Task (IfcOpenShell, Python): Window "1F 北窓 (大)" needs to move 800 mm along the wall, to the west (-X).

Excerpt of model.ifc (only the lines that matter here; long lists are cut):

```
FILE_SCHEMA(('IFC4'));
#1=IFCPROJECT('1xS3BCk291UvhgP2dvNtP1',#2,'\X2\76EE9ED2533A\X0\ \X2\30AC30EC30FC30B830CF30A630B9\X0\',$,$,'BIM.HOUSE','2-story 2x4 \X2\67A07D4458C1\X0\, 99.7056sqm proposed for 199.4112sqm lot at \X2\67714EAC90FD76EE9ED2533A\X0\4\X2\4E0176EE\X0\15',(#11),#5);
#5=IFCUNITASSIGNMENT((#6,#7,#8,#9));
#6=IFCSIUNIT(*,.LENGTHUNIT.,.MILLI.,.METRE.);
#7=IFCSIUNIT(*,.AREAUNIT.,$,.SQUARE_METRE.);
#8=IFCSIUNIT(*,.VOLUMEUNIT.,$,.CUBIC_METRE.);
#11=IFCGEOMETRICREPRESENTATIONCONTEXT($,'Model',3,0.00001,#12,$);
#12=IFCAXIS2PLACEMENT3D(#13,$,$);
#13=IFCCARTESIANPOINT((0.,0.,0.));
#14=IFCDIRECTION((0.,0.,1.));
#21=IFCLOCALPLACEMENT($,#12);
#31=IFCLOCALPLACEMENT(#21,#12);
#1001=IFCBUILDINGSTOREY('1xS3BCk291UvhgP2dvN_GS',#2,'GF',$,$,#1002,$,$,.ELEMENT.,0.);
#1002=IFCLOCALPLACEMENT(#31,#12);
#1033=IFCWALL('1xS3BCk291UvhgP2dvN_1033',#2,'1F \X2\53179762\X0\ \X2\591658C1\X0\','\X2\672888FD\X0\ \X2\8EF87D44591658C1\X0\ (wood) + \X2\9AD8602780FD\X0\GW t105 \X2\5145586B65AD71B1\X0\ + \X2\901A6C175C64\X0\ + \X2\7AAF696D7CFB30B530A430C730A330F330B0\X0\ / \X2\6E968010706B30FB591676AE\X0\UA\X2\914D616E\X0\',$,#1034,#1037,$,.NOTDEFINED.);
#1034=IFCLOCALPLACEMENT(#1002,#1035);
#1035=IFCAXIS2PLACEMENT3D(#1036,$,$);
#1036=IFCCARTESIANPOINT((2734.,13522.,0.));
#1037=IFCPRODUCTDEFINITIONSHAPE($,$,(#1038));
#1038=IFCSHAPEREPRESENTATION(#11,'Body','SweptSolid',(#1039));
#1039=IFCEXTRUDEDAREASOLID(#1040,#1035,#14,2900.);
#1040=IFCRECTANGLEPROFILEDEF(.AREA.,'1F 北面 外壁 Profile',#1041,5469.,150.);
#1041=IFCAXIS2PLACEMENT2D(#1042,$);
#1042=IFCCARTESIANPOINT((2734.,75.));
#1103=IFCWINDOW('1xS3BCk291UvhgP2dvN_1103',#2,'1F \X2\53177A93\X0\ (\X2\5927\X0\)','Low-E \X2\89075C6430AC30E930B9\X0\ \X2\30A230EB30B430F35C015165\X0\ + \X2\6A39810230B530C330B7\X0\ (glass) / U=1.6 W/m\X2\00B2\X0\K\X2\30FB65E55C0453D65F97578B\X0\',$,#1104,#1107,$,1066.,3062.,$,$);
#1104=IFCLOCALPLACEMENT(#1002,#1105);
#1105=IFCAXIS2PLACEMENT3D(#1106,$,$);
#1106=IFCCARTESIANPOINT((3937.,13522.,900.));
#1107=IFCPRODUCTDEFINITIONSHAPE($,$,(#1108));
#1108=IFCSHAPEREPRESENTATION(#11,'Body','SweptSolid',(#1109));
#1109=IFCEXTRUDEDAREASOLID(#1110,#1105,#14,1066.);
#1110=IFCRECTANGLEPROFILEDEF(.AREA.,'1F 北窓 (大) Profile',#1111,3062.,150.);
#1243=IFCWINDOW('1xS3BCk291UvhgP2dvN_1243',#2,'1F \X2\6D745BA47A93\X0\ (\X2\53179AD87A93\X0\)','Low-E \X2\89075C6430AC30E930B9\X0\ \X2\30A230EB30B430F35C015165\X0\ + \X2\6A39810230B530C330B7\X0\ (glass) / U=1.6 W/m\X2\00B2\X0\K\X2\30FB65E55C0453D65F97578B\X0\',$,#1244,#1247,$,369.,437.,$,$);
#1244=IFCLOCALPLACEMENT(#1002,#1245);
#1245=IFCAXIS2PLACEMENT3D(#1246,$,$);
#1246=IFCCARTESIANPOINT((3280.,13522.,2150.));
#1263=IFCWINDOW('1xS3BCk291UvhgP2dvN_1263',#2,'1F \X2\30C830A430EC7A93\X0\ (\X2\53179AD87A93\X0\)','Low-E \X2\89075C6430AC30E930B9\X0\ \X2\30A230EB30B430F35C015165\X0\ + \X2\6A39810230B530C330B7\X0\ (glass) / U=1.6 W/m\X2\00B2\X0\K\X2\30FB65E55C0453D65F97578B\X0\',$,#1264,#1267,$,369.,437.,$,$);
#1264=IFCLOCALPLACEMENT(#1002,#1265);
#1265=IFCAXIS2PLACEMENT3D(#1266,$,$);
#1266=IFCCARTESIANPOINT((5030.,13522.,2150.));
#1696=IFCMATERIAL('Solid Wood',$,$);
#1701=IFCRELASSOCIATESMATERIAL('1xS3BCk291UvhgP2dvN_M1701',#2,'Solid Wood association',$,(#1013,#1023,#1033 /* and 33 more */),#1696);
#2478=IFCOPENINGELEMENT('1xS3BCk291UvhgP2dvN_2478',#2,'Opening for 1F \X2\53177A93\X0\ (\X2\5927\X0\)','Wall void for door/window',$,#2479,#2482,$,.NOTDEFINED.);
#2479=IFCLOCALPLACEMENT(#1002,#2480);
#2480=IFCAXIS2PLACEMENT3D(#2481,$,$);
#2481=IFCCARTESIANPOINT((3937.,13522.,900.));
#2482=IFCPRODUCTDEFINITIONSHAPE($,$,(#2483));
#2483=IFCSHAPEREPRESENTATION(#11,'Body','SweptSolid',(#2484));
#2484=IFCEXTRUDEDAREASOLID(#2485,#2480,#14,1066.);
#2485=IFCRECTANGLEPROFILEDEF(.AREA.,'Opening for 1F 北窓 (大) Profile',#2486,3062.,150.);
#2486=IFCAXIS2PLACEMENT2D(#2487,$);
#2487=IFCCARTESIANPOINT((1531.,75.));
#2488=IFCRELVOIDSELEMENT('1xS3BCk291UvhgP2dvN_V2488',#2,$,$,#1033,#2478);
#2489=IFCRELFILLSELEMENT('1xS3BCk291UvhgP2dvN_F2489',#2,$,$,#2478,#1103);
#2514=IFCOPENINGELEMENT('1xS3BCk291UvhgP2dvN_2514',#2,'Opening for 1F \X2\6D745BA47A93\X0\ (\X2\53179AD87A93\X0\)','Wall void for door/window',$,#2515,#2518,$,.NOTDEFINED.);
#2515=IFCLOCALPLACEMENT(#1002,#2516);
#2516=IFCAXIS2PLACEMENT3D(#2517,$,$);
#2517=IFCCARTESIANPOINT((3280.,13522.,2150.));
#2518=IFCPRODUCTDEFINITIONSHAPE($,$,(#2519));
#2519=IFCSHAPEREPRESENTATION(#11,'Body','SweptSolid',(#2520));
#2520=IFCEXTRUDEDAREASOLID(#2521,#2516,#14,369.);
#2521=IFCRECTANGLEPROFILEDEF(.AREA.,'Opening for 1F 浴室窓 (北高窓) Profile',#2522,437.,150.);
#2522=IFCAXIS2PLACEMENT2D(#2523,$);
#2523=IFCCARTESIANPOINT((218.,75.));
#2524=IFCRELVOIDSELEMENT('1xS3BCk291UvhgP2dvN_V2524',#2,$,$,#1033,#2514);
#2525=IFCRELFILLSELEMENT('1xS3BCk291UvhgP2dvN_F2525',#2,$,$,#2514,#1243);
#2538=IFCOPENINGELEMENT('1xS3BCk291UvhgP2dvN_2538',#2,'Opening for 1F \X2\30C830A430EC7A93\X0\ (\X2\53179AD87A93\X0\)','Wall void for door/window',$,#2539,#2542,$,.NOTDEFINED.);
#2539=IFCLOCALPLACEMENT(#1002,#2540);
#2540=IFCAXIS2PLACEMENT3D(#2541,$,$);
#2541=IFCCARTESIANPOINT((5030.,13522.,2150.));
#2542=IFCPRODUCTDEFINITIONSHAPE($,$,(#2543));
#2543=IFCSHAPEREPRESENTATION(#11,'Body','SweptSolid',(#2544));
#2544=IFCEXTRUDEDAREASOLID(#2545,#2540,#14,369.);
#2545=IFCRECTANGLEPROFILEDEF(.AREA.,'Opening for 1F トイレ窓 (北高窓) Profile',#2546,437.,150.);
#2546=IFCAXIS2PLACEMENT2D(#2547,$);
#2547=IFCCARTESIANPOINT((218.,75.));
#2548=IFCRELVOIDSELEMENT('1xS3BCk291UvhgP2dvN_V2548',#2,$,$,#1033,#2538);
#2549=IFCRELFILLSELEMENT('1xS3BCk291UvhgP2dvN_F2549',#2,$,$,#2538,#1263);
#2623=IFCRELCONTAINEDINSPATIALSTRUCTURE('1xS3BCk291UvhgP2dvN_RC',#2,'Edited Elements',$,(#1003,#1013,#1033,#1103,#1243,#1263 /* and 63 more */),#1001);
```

```python
import ifcopenshell
import ifcopenshell.api.geometry
import ifcopenshell.util.placement

model = ifcopenshell.open("model.ifc")

window = model.by_guid("1xS3BCk291UvhgP2dvN_1103")
opening = window.FillsVoids[0].RelatingOpeningElement
wall = opening.VoidsElements[0].RelatingBuildingElement

wall_matrix = ifcopenshell.util.placement.get_local_placement(wall.ObjectPlacement)
shift = wall_matrix[:3, 0] * -800.0
before = ifcopenshell.util.placement.get_local_placement(window.ObjectPlacement)[:3, 3].copy()

# The window is not placed relative to its opening, so move both.
for product in (opening, window):
    matrix = ifcopenshell.util.placement.get_local_placement(product.ObjectPlacement)
    matrix[:3, 3] += shift
    ifcopenshell.api.geometry.edit_object_placement(model, product=product, matrix=matrix, is_si=False)

after = ifcopenshell.util.placement.get_local_placement(window.ObjectPlacement)[:3, 3]
print("window moved by", (after - before).round(3) + 0.0)

model.write("model_edited.ifc")
```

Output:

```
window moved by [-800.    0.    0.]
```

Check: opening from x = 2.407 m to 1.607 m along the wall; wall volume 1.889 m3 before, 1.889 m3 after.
